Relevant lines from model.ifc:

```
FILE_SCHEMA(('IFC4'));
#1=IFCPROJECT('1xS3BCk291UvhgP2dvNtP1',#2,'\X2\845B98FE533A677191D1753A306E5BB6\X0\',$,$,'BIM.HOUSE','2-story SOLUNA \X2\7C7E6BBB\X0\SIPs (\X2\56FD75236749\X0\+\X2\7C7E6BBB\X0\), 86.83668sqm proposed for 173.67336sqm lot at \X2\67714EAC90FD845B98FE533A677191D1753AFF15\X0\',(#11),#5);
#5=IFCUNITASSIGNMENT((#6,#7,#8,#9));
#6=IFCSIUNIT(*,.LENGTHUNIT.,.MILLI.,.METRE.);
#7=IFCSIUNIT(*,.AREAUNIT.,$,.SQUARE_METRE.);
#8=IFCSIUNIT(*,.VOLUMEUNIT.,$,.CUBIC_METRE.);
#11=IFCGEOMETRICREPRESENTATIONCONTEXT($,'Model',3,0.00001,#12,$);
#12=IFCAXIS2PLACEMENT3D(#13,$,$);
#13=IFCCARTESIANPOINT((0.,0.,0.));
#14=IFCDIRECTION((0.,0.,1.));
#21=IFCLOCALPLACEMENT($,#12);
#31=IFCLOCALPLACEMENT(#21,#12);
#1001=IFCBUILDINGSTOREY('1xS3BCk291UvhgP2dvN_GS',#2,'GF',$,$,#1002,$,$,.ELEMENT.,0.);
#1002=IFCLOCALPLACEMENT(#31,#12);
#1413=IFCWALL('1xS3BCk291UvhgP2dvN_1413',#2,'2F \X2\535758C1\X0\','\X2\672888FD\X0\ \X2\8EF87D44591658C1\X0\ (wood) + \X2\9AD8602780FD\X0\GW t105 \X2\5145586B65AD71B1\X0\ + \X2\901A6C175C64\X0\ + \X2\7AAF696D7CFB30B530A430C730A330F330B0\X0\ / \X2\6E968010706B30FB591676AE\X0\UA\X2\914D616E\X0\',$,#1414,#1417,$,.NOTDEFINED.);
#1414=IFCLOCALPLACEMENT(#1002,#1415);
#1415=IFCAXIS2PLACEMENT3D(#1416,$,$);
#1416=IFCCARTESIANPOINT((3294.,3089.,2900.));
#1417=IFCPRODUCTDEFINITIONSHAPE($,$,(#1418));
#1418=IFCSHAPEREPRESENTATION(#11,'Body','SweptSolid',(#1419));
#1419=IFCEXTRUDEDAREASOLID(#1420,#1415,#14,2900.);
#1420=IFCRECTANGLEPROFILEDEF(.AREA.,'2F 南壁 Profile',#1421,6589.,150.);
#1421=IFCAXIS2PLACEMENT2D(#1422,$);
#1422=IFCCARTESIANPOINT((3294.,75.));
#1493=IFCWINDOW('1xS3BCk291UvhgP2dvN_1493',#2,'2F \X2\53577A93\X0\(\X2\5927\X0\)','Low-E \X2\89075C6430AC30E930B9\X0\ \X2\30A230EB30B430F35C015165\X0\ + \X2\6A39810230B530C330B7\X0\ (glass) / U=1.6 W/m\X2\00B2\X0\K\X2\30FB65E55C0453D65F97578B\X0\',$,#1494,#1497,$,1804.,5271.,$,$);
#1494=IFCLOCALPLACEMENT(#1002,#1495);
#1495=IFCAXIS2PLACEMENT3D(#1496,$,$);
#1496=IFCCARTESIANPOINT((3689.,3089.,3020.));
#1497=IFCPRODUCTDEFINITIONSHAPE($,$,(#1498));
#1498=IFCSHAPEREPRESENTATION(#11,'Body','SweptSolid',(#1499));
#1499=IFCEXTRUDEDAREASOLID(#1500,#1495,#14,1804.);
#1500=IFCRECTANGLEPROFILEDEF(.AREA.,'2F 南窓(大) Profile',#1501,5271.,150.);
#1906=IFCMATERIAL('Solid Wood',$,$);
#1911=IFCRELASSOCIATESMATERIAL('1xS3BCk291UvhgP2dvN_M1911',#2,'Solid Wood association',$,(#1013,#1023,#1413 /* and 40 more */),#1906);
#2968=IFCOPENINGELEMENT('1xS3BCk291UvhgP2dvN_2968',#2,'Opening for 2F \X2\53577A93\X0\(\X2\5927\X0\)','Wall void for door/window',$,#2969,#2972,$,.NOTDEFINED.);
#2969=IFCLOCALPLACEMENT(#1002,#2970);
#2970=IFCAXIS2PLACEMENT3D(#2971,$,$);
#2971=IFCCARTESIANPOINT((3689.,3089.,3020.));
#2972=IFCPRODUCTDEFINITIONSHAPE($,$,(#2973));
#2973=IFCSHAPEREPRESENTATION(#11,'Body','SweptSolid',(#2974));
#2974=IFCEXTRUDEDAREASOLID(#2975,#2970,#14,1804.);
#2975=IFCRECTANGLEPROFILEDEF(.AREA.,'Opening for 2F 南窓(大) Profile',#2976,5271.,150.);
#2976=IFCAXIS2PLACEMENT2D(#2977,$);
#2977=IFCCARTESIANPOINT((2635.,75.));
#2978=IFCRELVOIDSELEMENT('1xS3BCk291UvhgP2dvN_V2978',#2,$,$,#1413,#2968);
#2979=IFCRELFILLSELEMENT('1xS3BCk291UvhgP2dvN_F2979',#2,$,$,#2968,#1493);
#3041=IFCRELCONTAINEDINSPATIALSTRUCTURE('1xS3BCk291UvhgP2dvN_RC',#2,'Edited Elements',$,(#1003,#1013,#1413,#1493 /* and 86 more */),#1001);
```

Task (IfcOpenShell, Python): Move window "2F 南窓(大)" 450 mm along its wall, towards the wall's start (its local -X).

```python
import ifcopenshell
import ifcopenshell.api.geometry
import ifcopenshell.util.placement
import ifcopenshell.util.unit

model = ifcopenshell.open("model.ifc")
unit_scale = ifcopenshell.util.unit.calculate_unit_scale(model)

window = model.by_id(1493)
opening = window.FillsVoids[0].RelatingOpeningElement
wall = opening.VoidsElements[0].RelatingBuildingElement

wall_matrix = ifcopenshell.util.placement.get_local_placement(wall.ObjectPlacement)
shift = wall_matrix[:3, 0] * -0.45 / unit_scale
before = ifcopenshell.util.placement.get_local_placement(window.ObjectPlacement)[:3, 3].copy()

# The window is not placed relative to its opening, so move both.
for product in (opening, window):
    matrix = ifcopenshell.util.placement.get_local_placement(product.ObjectPlacement)
    matrix[:3, 3] += shift
    ifcopenshell.api.geometry.edit_object_placement(model, product=product, matrix=matrix, is_si=False)

after = ifcopenshell.util.placement.get_local_placement(window.ObjectPlacement)[:3, 3]
print("window moved by", (after - before).round(3) + 0.0)

model.write("model_rev.ifc")
```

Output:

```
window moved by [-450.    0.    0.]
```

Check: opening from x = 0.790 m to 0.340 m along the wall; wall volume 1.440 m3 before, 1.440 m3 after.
